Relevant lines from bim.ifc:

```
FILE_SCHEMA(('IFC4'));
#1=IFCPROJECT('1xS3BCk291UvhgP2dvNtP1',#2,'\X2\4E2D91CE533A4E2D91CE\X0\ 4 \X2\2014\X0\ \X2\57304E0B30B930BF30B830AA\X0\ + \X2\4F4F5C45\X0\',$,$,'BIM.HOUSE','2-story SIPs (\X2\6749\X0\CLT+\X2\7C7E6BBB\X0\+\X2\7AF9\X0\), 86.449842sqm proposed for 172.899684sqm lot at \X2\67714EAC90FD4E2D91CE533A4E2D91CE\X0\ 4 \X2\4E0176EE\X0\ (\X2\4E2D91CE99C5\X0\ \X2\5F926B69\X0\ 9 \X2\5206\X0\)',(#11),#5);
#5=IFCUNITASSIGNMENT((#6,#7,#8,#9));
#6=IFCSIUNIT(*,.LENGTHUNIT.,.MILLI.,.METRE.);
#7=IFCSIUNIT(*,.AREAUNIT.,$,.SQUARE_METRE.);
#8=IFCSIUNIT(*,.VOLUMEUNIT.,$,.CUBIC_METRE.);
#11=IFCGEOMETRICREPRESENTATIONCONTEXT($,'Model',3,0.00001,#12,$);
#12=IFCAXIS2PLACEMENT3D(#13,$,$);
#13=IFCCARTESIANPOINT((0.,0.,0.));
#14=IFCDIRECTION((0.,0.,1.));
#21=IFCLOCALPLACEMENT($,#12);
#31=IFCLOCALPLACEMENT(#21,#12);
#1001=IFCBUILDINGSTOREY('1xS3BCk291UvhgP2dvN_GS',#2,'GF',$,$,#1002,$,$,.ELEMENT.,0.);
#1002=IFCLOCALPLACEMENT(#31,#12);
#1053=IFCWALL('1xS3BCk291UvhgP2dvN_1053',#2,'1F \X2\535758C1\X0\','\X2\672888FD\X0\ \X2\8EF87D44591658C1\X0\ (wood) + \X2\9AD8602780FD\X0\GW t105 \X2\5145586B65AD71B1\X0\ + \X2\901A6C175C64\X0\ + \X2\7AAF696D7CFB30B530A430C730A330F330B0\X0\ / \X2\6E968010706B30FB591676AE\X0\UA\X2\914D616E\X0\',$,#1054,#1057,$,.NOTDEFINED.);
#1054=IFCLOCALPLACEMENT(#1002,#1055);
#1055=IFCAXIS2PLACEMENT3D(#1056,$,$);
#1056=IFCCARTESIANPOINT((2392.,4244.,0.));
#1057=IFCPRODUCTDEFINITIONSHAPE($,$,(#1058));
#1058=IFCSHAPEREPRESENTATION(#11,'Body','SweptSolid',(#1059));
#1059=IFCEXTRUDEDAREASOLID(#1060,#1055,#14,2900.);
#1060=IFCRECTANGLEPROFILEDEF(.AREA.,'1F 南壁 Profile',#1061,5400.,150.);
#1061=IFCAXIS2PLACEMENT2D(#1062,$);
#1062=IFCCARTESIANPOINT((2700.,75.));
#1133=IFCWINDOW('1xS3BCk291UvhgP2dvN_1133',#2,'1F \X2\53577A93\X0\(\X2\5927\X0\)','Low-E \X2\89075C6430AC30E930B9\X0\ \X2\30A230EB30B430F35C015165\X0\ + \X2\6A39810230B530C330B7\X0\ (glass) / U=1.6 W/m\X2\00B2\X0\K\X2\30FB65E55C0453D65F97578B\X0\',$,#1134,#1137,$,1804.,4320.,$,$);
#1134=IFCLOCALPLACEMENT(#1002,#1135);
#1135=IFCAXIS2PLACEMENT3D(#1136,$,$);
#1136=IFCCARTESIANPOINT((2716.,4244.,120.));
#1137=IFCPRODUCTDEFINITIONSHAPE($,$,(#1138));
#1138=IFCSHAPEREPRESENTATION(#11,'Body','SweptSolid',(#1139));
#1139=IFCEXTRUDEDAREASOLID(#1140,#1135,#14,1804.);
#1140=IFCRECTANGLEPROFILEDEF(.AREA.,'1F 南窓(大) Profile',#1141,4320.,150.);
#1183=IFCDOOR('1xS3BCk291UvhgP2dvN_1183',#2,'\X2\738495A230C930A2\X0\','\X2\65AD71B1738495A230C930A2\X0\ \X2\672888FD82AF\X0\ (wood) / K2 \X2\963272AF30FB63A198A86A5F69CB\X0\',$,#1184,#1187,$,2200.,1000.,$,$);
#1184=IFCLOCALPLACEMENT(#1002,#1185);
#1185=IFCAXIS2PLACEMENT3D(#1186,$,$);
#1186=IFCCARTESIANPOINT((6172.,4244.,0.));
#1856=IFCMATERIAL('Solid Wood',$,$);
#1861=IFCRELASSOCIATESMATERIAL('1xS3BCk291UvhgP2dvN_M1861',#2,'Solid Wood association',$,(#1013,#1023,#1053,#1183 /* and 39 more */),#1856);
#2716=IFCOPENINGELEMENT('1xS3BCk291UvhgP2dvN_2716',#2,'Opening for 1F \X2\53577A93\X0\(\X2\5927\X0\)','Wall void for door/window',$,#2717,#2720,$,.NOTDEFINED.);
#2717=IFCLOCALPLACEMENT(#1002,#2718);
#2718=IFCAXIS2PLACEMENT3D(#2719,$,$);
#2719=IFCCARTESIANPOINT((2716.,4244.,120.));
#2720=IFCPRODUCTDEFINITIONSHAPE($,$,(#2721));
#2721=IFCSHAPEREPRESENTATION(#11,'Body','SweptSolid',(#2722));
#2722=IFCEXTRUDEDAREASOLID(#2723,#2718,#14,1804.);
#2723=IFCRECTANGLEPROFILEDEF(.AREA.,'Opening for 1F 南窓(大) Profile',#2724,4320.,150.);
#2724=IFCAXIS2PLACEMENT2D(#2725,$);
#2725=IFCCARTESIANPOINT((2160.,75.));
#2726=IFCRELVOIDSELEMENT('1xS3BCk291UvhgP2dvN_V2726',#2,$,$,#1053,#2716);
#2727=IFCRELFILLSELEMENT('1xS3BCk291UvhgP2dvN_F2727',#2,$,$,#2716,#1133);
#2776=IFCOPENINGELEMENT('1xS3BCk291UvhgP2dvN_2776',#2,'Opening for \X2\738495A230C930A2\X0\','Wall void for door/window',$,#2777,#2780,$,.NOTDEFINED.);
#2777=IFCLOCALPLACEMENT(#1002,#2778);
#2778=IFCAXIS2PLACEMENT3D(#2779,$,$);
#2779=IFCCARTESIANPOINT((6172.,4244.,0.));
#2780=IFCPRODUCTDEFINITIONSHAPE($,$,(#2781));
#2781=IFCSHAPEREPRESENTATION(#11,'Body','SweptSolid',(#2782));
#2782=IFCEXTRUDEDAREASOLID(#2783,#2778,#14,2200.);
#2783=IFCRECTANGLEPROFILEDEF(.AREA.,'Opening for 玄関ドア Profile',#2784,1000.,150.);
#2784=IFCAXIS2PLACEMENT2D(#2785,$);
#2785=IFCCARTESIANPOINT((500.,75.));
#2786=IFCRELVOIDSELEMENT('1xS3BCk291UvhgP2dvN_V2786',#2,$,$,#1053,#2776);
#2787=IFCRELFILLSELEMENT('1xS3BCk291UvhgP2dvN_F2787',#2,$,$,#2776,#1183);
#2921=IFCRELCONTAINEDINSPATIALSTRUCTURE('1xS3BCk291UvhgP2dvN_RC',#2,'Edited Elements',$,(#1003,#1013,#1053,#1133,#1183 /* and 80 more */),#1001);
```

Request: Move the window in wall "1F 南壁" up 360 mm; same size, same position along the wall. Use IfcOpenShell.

```python
import numpy as np
import ifcopenshell
import ifcopenshell.api.geometry
import ifcopenshell.util.placement
import ifcopenshell.util.unit

model = ifcopenshell.open("bim.ifc")
unit_scale = ifcopenshell.util.unit.calculate_unit_scale(model)

window = model.by_guid("1xS3BCk291UvhgP2dvN_1133")
opening = window.FillsVoids[0].RelatingOpeningElement
dz = 360.0

shift = np.array([0.0, 0.0, dz])
# The window is not placed relative to its opening, so move both.
for product in (opening, window):
    matrix = ifcopenshell.util.placement.get_local_placement(product.ObjectPlacement)
    matrix[:3, 3] += shift
    ifcopenshell.api.geometry.edit_object_placement(model, product=product, matrix=matrix, is_si=False)

print(f"moved by {dz * unit_scale:+.3f} m")

model.write("bim_v2.ifc")
```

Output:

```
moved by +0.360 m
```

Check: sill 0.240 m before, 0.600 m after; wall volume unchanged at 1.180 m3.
